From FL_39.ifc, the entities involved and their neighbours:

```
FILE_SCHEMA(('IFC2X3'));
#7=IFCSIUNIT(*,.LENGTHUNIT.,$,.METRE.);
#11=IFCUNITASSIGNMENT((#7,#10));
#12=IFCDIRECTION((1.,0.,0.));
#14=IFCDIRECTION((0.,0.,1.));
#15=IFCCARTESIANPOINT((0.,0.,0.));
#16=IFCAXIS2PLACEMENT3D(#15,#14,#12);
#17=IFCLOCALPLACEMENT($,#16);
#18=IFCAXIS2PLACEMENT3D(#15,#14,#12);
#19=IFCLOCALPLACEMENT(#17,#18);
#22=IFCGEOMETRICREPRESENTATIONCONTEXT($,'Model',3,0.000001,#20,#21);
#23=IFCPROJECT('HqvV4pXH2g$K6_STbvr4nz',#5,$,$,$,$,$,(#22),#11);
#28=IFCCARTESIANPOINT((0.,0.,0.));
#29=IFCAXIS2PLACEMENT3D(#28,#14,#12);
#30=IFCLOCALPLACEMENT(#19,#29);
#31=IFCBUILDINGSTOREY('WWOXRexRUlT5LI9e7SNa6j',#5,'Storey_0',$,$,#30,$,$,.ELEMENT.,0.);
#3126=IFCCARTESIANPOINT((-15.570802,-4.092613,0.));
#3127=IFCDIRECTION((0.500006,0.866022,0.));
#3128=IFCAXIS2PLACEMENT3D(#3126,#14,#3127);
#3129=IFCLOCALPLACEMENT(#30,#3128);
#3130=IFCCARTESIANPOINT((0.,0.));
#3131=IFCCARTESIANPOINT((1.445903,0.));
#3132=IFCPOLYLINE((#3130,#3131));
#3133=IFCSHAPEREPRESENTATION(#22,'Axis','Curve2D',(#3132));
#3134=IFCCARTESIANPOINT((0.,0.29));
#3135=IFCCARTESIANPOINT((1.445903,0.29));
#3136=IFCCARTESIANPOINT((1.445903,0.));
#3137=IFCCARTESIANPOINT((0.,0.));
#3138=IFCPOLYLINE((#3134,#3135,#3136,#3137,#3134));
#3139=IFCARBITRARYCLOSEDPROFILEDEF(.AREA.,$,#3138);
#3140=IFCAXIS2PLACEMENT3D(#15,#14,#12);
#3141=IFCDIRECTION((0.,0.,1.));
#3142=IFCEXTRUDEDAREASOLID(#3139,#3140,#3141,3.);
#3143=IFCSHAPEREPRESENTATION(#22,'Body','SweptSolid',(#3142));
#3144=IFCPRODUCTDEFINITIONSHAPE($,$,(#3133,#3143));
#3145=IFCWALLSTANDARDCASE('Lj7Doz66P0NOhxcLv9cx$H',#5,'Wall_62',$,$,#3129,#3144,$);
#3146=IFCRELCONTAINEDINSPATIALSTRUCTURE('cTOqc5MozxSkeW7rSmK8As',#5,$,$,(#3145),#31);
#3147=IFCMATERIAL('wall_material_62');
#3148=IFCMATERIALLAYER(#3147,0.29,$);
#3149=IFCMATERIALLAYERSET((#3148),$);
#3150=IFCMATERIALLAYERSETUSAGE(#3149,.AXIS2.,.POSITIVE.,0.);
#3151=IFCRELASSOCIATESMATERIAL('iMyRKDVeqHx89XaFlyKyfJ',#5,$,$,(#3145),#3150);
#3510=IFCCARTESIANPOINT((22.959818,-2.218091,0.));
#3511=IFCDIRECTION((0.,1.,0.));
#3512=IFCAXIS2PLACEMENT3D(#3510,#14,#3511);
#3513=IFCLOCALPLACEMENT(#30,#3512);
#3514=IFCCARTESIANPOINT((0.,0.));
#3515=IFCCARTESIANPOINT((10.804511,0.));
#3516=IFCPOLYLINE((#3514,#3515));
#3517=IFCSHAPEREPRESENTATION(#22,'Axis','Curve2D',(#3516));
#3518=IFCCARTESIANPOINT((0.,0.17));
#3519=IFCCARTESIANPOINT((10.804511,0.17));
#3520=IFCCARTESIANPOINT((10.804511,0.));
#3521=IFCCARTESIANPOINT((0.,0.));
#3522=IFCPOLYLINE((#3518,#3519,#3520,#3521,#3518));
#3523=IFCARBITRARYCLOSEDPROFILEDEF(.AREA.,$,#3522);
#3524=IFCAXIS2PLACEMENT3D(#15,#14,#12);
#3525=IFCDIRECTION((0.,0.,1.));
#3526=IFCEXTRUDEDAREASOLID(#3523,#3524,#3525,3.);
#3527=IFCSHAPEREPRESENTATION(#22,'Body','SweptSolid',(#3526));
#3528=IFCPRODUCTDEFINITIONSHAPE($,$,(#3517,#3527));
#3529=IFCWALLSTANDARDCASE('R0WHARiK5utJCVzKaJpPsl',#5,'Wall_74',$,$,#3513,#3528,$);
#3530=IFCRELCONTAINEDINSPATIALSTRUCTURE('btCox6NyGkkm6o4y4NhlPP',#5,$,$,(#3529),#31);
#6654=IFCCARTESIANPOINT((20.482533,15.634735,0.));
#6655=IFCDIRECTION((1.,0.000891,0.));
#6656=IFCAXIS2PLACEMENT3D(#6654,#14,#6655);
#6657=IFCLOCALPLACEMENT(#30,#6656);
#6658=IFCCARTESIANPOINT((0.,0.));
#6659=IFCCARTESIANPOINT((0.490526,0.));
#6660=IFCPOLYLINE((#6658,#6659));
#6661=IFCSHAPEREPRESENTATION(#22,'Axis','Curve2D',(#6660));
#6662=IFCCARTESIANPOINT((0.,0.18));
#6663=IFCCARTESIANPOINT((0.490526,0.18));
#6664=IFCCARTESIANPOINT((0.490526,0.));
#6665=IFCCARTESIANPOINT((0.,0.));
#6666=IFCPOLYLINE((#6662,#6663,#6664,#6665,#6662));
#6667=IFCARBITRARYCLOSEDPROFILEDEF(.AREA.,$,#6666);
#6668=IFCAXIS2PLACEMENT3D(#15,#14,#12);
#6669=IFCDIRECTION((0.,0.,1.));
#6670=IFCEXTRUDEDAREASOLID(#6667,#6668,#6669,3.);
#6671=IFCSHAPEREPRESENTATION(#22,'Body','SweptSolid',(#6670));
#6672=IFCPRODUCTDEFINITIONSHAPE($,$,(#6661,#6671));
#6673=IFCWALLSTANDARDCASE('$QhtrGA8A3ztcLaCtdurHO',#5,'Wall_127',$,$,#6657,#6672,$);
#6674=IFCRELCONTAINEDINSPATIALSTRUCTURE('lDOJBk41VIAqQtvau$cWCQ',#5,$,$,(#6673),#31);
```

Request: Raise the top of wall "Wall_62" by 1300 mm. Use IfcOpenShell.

```python
import ifcopenshell
import ifcopenshell.geom
import ifcopenshell.util.shape
import ifcopenshell.util.unit

model = ifcopenshell.open("FL_39.ifc")
unit_scale = ifcopenshell.util.unit.calculate_unit_scale(model)
settings = ifcopenshell.geom.settings()


def volume(element):
    """Net volume in cubic metres, openings subtracted."""
    shape = ifcopenshell.geom.create_shape(settings, element)
    return ifcopenshell.util.shape.get_volume(shape.geometry)


wall = model.by_guid("Lj7Doz66P0NOhxcLv9cx$H")
before = volume(wall)

body = next(r for r in wall.Representation.Representations if r.RepresentationIdentifier == "Body")
solid = body.Items[0]
old_height = solid.Depth
solid.Depth += 1.3 / unit_scale
after = volume(wall)

print(f"height {old_height:g} -> {solid.Depth:g}, volume {before:.3f} -> {after:.3f} m3")

model.write("FL_39_rev.ifc")
```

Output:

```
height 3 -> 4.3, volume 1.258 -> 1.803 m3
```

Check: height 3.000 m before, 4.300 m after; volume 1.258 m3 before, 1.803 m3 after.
